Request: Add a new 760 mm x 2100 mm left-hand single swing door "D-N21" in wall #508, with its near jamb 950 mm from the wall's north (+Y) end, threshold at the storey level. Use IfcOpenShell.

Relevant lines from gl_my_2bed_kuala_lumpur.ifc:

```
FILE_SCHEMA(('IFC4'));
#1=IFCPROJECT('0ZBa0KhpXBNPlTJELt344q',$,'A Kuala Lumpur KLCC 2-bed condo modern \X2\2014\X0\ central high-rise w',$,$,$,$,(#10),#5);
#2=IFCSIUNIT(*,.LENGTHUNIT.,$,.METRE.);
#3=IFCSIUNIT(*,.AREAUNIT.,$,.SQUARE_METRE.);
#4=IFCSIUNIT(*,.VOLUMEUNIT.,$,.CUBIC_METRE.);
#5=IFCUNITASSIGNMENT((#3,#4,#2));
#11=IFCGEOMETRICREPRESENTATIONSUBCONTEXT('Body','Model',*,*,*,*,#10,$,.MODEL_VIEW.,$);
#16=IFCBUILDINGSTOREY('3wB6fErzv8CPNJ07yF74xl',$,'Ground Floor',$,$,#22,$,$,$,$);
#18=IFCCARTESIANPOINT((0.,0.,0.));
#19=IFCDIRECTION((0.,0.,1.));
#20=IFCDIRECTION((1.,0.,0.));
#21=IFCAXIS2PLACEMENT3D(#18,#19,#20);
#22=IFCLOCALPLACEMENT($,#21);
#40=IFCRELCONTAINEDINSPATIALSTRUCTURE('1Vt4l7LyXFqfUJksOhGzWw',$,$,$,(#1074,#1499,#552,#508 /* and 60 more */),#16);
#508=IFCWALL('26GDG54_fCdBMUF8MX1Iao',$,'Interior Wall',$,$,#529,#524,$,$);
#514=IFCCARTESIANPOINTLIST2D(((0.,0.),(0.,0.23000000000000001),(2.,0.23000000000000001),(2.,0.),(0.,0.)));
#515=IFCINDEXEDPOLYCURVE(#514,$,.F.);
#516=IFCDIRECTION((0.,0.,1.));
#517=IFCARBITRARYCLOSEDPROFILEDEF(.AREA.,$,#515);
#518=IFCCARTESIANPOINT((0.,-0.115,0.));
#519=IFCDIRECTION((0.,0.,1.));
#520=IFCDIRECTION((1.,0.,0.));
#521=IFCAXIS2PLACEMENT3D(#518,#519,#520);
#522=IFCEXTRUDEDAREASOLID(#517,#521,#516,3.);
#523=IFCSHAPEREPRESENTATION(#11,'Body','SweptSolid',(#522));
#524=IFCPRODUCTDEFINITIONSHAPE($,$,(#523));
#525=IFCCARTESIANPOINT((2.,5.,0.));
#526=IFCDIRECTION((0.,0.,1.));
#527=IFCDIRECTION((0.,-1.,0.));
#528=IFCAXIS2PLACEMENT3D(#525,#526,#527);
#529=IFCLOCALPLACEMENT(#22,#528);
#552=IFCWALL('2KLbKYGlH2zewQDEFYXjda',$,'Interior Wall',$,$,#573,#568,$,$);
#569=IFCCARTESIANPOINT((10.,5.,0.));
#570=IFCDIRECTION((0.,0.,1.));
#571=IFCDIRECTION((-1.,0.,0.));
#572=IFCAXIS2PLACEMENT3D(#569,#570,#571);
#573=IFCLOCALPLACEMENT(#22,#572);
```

```python
import numpy as np
import ifcopenshell
import ifcopenshell.api.feature
import ifcopenshell.api.geometry
import ifcopenshell.api.root
import ifcopenshell.api.spatial
import ifcopenshell.geom
import ifcopenshell.util.element
import ifcopenshell.util.placement
import ifcopenshell.util.representation
import ifcopenshell.util.shape
import ifcopenshell.util.unit

model = ifcopenshell.open("gl_my_2bed_kuala_lumpur.ifc")
unit_scale = ifcopenshell.util.unit.calculate_unit_scale(model)
settings = ifcopenshell.geom.settings()


def volume(element):
    """Net volume in cubic metres, openings subtracted."""
    shape = ifcopenshell.geom.create_shape(settings, element)
    return ifcopenshell.util.shape.get_volume(shape.geometry)


wall = model.by_guid("26GDG54_fCdBMUF8MX1Iao")
storey = ifcopenshell.util.element.get_container(wall, ifc_class="IfcBuildingStorey")
context = ifcopenshell.util.representation.get_context(model, "Model", "Body", "MODEL_VIEW")
before = volume(wall)

width, height, from_end, sill = 0.76, 2.1, 0.95, 0.0  # metres

# The wall runs along its own X axis, and the end named is its -X end.
wall_shape = ifcopenshell.geom.create_shape(settings, wall)
x, y, z = ifcopenshell.util.shape.get_vertices(wall_shape.geometry).T
start = x.min() + from_end
face, thickness = float(y.min()), float(y.max() - y.min())
wall_matrix = ifcopenshell.util.placement.get_local_placement(wall.ObjectPlacement)
level = ifcopenshell.util.placement.get_local_placement(storey.ObjectPlacement)[2, 3]


def in_wall(x, y):
    """Placement at x, y metres in the wall's axes, at sill height."""
    matrix = wall_matrix.copy()
    matrix[:, 3] = wall_matrix @ np.array([x / unit_scale, y / unit_scale, 0.0, 1.0])
    matrix[2, 3] = level + sill / unit_scale
    return matrix


# Opening: a box that overshoots both wall faces by 50 mm.
opening = ifcopenshell.api.root.create_entity(model, ifc_class="IfcOpeningElement", predefined_type="OPENING")
box = ifcopenshell.api.geometry.add_wall_representation(
    model, context=context, length=width, height=height, thickness=thickness + 0.1
)
ifcopenshell.api.geometry.assign_representation(model, product=opening, representation=box)
ifcopenshell.api.geometry.edit_object_placement(model, product=opening, matrix=in_wall(start, face - 0.05), is_si=False)
ifcopenshell.api.feature.add_feature(model, feature=opening, element=wall)

door = ifcopenshell.api.root.create_entity(model, ifc_class="IfcDoor", name="D-N21", predefined_type="DOOR")
door.OverallWidth, door.OverallHeight = width / unit_scale, height / unit_scale
door.OperationType = "SINGLE_SWING_LEFT"
body = ifcopenshell.api.geometry.add_door_representation(
    model,
    context=context,
    overall_width=door.OverallWidth,
    overall_height=door.OverallHeight,
    operation_type="SINGLE_SWING_LEFT",
    lining_properties={"LiningDepth": thickness / unit_scale, "ThresholdDepth": thickness / unit_scale},
)
ifcopenshell.api.geometry.assign_representation(model, product=door, representation=body)
ifcopenshell.api.spatial.assign_container(model, products=[door], relating_structure=storey)
ifcopenshell.api.feature.add_filling(model, opening=opening, element=door)

# The lining spans the wall, so the door starts at the wall face.
ifcopenshell.api.geometry.edit_object_placement(model, product=door, matrix=in_wall(start, face), is_si=False)

after = volume(wall)

print(f"wall volume {before:.3f} -> {after:.3f} m3")

model.write("gl_my_2bed_kuala_lumpur-out.ifc")
```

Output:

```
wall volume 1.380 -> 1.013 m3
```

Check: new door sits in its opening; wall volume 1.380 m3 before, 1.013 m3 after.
